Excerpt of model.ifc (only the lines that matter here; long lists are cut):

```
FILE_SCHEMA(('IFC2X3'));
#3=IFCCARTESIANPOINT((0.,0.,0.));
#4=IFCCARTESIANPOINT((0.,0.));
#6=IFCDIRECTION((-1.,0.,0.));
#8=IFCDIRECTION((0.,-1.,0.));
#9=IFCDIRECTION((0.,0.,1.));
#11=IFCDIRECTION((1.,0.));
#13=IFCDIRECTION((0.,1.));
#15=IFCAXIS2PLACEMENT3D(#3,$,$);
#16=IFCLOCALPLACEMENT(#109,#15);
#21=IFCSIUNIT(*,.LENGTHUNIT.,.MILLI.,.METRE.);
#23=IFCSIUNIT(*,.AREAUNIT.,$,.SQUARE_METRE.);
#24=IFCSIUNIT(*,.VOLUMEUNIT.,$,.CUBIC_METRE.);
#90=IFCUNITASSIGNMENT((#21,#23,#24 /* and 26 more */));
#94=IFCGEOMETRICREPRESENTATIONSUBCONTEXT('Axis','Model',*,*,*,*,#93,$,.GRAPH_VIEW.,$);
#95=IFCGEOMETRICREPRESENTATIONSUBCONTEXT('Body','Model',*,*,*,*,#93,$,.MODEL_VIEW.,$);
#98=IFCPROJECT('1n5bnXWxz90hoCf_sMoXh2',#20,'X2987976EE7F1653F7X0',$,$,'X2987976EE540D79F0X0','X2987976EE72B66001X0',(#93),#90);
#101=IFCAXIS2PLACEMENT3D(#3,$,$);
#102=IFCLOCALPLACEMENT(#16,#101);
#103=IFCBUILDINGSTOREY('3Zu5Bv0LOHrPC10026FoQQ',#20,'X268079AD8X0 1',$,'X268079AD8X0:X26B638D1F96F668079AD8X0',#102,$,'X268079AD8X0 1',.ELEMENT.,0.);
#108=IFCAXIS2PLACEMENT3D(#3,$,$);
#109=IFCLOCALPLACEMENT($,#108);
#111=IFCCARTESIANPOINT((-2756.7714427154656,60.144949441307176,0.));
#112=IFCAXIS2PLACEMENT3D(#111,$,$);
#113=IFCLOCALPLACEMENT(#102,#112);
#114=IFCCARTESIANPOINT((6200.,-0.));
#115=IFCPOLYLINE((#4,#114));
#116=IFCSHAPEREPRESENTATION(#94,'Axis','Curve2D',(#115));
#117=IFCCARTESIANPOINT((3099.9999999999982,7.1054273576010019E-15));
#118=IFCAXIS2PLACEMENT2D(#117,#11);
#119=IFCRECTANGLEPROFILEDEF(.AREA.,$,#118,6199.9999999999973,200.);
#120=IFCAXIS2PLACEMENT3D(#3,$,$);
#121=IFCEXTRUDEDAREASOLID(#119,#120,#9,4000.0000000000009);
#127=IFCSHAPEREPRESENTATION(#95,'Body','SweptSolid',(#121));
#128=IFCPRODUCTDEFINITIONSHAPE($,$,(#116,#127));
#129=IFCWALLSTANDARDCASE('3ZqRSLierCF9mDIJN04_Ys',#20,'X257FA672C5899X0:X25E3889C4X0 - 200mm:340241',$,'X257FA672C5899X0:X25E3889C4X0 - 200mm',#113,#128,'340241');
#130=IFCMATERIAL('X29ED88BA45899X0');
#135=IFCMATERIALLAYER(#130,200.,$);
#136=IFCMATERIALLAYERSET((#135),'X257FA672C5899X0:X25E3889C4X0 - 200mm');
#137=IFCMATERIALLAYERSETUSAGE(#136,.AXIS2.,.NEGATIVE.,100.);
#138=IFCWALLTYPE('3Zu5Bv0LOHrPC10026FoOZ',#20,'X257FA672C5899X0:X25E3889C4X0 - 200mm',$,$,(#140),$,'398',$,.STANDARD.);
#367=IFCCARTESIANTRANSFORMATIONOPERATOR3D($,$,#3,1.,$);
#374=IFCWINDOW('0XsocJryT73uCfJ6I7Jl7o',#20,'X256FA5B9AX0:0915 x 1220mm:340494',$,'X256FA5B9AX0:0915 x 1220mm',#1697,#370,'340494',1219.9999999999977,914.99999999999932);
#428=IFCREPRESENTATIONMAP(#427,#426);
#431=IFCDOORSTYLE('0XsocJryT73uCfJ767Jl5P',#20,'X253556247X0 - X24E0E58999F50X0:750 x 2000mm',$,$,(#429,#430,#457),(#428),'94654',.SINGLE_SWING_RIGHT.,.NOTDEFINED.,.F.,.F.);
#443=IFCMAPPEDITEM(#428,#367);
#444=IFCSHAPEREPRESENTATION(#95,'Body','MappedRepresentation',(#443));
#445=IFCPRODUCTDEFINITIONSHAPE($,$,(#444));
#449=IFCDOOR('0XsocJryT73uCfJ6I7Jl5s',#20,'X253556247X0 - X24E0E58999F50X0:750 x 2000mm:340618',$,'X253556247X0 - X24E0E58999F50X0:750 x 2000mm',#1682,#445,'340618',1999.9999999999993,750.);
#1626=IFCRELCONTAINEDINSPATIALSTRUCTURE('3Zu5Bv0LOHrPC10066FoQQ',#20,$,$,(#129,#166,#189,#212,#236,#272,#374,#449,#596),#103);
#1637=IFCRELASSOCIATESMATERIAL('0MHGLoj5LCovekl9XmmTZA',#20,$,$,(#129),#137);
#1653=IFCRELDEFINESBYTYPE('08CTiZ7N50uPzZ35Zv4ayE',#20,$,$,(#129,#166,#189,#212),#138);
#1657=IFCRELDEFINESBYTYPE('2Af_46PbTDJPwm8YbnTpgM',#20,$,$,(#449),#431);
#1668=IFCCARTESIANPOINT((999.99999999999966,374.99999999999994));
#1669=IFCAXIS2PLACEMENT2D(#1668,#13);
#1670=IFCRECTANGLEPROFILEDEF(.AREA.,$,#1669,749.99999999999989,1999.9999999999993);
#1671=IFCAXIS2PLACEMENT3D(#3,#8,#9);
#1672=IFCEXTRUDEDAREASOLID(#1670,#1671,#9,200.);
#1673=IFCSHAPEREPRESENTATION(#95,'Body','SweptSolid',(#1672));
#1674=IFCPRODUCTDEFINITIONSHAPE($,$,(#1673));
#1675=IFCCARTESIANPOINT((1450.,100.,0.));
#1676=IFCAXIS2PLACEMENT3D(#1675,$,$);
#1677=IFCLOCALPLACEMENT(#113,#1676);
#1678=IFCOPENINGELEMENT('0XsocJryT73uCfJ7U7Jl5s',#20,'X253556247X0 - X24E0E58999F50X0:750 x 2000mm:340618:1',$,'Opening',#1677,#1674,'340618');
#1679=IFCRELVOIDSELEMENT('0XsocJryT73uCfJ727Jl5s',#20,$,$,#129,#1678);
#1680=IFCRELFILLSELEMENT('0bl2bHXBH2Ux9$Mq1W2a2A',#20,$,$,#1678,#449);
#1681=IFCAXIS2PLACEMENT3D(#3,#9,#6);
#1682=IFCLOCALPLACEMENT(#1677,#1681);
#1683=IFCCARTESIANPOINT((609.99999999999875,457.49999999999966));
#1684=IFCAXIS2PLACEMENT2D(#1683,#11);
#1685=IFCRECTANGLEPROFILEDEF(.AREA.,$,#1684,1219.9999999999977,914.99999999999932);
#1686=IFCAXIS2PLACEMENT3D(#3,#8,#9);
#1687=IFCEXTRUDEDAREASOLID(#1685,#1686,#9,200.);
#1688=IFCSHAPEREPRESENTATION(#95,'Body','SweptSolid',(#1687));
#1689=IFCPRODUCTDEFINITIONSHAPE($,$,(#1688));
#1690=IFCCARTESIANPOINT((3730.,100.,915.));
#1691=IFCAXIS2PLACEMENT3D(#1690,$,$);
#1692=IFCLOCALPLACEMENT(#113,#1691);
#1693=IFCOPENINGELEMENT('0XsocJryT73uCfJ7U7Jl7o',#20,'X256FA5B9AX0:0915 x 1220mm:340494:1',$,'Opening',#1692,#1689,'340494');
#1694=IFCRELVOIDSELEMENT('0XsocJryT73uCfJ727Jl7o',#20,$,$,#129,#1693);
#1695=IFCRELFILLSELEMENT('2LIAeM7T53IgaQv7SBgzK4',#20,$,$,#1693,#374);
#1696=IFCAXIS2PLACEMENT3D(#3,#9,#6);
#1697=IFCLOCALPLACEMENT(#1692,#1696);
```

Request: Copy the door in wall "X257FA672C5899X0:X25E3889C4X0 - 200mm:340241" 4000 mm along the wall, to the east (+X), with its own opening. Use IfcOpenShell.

```python
import ifcopenshell
import ifcopenshell.api.feature
import ifcopenshell.api.geometry
import ifcopenshell.api.root
import ifcopenshell.geom
import ifcopenshell.util.element
import ifcopenshell.util.placement
import ifcopenshell.util.shape
import ifcopenshell.util.unit

model = ifcopenshell.open("model.ifc")
unit_scale = ifcopenshell.util.unit.calculate_unit_scale(model)
settings = ifcopenshell.geom.settings()


def volume(element):
    """Net volume in cubic metres, openings subtracted."""
    shape = ifcopenshell.geom.create_shape(settings, element)
    return ifcopenshell.util.shape.get_volume(shape.geometry)


def reuse_history(source, copy):
    """copy_class also copies each property set's owner history, people and application; keep the originals."""
    for rel in copy.IsDefinedBy:
        if rel.is_a("IfcRelDefinesByProperties") and (history := rel.RelatingPropertyDefinition.OwnerHistory):
            rel.RelatingPropertyDefinition.OwnerHistory = source.OwnerHistory
            ifcopenshell.util.element.remove_deep2(model, history)


door = model.by_guid("0XsocJryT73uCfJ6I7Jl5s")
opening = door.FillsVoids[0].RelatingOpeningElement
wall = opening.VoidsElements[0].RelatingBuildingElement
before = volume(wall)
shift = ifcopenshell.util.placement.get_local_placement(wall.ObjectPlacement)[:3, 0] * 4 / unit_scale

# copy_class copies the void relationship, type, container and properties, but no geometry.
new_opening = ifcopenshell.api.root.copy_class(model, product=opening)
new_opening.Representation = ifcopenshell.util.element.copy_deep(
    model, opening.Representation, exclude=["IfcGeometricRepresentationContext", "IfcRepresentationMap"]
)
new_opening.Name = "X253556247X0 - X24E0E58999F50X0:750 x 2000mm"
new_opening.Tag = None
new_door = ifcopenshell.api.root.copy_class(model, product=door)
new_door.Representation = ifcopenshell.util.element.copy_deep(
    model, door.Representation, exclude=["IfcGeometricRepresentationContext", "IfcRepresentationMap"]
)
new_door.Name = "X253556247X0 - X24E0E58999F50X0:750 x 2000mm"
new_door.Tag = None
reuse_history(door, new_door)
fills = ifcopenshell.api.feature.add_filling(model, opening=new_opening, element=new_door)
fills.OwnerHistory = new_door.OwnerHistory  # required in IFC2X3

for old, new in ((opening, new_opening), (door, new_door)):
    matrix = ifcopenshell.util.placement.get_local_placement(old.ObjectPlacement)
    matrix[:3, 3] += shift
    ifcopenshell.api.geometry.edit_object_placement(model, product=new, matrix=matrix, is_si=False)

after = volume(wall)

print(f"wall volume {before:.3f} -> {after:.3f} m3")

model.write("model_updated.ifc")
```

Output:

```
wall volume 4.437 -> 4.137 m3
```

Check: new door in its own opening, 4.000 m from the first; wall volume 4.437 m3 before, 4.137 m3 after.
